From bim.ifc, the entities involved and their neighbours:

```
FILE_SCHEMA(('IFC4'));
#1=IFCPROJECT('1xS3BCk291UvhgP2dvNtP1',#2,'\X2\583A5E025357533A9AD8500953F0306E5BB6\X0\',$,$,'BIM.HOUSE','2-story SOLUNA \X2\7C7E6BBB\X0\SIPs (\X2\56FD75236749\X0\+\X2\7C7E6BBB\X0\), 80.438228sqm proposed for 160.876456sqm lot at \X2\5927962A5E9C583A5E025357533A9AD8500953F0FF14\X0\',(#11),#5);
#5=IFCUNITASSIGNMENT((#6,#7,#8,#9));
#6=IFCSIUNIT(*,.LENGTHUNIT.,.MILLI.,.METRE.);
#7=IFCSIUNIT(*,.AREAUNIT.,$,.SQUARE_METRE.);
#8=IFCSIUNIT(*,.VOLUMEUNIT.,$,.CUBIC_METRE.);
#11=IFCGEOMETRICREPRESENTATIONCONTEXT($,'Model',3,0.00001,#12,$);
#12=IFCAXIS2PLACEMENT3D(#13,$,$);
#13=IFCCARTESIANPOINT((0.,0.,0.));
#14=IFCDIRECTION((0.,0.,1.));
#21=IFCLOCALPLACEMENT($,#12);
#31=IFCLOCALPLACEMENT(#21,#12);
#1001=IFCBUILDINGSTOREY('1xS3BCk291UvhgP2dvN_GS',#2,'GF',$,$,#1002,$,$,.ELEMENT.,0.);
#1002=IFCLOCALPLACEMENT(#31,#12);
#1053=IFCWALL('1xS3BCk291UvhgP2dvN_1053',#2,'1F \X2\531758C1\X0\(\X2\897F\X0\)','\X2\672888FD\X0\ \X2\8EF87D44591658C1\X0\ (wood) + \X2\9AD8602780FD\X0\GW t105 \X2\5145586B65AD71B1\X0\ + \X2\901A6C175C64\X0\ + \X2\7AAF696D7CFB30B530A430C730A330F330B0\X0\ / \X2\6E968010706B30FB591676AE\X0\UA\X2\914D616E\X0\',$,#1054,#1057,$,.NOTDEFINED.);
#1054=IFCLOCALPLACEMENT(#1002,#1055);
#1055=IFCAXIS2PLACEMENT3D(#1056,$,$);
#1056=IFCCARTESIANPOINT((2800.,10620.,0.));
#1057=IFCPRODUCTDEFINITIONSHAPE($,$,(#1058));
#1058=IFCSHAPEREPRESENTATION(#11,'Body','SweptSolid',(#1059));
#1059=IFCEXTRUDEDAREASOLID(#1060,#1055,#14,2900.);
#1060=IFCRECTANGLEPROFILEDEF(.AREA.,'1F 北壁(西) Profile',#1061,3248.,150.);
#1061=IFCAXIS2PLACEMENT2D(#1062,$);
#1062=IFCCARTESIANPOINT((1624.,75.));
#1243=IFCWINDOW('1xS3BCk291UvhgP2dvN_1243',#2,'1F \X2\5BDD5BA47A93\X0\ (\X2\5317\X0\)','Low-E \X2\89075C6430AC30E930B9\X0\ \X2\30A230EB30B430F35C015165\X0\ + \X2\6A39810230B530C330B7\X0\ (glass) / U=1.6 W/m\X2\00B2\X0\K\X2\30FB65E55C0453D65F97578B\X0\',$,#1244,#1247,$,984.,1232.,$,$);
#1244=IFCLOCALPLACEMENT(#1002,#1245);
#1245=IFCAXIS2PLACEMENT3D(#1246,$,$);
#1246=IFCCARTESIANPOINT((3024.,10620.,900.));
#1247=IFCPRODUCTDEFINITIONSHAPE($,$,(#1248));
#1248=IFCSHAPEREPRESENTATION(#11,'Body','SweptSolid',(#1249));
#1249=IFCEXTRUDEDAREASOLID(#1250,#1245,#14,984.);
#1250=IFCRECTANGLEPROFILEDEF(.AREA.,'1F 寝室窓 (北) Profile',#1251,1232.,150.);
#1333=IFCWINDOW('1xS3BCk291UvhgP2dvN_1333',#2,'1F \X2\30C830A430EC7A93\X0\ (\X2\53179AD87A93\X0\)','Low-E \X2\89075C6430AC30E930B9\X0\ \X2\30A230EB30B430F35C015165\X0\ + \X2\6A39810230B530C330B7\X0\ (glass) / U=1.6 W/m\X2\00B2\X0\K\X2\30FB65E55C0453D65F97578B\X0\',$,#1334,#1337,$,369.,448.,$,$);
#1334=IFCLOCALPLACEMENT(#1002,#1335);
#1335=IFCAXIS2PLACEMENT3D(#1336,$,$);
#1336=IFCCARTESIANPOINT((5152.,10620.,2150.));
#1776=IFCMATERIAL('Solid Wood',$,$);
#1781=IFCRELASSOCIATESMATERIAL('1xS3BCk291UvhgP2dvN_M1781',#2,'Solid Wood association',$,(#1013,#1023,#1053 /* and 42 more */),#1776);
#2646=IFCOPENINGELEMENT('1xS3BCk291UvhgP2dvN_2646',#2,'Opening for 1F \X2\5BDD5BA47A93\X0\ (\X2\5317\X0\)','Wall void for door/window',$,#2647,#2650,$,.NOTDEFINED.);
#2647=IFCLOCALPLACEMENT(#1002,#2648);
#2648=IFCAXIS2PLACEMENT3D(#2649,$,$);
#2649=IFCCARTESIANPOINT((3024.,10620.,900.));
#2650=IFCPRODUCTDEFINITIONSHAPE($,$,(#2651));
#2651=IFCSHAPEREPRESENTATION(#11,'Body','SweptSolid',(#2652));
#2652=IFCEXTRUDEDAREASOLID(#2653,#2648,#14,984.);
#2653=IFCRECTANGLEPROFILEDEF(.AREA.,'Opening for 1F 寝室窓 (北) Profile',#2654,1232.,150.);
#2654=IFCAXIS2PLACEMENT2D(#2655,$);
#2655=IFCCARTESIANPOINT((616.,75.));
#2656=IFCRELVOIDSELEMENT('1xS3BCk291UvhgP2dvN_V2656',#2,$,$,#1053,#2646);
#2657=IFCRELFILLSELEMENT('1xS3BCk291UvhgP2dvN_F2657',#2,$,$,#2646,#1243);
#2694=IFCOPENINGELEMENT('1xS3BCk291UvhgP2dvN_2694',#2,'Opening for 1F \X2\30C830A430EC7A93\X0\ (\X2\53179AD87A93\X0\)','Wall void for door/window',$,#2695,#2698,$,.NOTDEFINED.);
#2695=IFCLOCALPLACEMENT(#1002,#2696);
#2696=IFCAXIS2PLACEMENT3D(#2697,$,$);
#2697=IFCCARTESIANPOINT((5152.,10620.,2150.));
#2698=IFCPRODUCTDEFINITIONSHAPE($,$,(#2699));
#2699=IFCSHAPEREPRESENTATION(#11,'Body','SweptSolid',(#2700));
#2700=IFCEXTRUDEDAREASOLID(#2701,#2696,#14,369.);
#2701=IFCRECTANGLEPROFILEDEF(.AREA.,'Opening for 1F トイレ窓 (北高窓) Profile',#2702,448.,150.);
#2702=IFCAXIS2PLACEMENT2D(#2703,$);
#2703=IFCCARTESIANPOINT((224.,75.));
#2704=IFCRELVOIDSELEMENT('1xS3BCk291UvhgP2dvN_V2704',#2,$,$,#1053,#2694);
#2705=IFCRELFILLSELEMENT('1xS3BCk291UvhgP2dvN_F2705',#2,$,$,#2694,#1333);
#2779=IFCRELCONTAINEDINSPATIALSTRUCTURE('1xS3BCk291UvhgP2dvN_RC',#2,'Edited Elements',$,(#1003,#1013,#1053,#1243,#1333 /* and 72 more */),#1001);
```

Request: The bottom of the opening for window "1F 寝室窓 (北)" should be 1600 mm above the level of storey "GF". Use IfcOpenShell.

```python
import numpy as np
import ifcopenshell
import ifcopenshell.api.geometry
import ifcopenshell.geom
import ifcopenshell.util.element
import ifcopenshell.util.placement
import ifcopenshell.util.shape
import ifcopenshell.util.unit

model = ifcopenshell.open("bim.ifc")
unit_scale = ifcopenshell.util.unit.calculate_unit_scale(model)

window = model.by_guid("1xS3BCk291UvhgP2dvN_1243")
opening = window.FillsVoids[0].RelatingOpeningElement
storey = ifcopenshell.util.element.get_container(window, ifc_class="IfcBuildingStorey")
level = ifcopenshell.util.placement.get_local_placement(storey.ObjectPlacement)[2, 3]

# The opening's origin need not be at the sill, so measure its lowest point.
shape = ifcopenshell.geom.create_shape(ifcopenshell.geom.settings(), opening)
bottom = ifcopenshell.util.shape.get_shape_bottom_elevation(shape, shape.geometry) / unit_scale
dz = level + 1.6 / unit_scale - bottom

shift = np.array([0.0, 0.0, dz])
# The window is not placed relative to its opening, so move both.
for product in (opening, window):
    matrix = ifcopenshell.util.placement.get_local_placement(product.ObjectPlacement)
    matrix[:3, 3] += shift
    ifcopenshell.api.geometry.edit_object_placement(model, product=product, matrix=matrix, is_si=False)

print(f"moved by {dz * unit_scale:+.3f} m")

model.write("bim_edited.ifc")
```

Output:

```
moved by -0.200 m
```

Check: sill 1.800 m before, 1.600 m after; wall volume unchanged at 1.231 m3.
